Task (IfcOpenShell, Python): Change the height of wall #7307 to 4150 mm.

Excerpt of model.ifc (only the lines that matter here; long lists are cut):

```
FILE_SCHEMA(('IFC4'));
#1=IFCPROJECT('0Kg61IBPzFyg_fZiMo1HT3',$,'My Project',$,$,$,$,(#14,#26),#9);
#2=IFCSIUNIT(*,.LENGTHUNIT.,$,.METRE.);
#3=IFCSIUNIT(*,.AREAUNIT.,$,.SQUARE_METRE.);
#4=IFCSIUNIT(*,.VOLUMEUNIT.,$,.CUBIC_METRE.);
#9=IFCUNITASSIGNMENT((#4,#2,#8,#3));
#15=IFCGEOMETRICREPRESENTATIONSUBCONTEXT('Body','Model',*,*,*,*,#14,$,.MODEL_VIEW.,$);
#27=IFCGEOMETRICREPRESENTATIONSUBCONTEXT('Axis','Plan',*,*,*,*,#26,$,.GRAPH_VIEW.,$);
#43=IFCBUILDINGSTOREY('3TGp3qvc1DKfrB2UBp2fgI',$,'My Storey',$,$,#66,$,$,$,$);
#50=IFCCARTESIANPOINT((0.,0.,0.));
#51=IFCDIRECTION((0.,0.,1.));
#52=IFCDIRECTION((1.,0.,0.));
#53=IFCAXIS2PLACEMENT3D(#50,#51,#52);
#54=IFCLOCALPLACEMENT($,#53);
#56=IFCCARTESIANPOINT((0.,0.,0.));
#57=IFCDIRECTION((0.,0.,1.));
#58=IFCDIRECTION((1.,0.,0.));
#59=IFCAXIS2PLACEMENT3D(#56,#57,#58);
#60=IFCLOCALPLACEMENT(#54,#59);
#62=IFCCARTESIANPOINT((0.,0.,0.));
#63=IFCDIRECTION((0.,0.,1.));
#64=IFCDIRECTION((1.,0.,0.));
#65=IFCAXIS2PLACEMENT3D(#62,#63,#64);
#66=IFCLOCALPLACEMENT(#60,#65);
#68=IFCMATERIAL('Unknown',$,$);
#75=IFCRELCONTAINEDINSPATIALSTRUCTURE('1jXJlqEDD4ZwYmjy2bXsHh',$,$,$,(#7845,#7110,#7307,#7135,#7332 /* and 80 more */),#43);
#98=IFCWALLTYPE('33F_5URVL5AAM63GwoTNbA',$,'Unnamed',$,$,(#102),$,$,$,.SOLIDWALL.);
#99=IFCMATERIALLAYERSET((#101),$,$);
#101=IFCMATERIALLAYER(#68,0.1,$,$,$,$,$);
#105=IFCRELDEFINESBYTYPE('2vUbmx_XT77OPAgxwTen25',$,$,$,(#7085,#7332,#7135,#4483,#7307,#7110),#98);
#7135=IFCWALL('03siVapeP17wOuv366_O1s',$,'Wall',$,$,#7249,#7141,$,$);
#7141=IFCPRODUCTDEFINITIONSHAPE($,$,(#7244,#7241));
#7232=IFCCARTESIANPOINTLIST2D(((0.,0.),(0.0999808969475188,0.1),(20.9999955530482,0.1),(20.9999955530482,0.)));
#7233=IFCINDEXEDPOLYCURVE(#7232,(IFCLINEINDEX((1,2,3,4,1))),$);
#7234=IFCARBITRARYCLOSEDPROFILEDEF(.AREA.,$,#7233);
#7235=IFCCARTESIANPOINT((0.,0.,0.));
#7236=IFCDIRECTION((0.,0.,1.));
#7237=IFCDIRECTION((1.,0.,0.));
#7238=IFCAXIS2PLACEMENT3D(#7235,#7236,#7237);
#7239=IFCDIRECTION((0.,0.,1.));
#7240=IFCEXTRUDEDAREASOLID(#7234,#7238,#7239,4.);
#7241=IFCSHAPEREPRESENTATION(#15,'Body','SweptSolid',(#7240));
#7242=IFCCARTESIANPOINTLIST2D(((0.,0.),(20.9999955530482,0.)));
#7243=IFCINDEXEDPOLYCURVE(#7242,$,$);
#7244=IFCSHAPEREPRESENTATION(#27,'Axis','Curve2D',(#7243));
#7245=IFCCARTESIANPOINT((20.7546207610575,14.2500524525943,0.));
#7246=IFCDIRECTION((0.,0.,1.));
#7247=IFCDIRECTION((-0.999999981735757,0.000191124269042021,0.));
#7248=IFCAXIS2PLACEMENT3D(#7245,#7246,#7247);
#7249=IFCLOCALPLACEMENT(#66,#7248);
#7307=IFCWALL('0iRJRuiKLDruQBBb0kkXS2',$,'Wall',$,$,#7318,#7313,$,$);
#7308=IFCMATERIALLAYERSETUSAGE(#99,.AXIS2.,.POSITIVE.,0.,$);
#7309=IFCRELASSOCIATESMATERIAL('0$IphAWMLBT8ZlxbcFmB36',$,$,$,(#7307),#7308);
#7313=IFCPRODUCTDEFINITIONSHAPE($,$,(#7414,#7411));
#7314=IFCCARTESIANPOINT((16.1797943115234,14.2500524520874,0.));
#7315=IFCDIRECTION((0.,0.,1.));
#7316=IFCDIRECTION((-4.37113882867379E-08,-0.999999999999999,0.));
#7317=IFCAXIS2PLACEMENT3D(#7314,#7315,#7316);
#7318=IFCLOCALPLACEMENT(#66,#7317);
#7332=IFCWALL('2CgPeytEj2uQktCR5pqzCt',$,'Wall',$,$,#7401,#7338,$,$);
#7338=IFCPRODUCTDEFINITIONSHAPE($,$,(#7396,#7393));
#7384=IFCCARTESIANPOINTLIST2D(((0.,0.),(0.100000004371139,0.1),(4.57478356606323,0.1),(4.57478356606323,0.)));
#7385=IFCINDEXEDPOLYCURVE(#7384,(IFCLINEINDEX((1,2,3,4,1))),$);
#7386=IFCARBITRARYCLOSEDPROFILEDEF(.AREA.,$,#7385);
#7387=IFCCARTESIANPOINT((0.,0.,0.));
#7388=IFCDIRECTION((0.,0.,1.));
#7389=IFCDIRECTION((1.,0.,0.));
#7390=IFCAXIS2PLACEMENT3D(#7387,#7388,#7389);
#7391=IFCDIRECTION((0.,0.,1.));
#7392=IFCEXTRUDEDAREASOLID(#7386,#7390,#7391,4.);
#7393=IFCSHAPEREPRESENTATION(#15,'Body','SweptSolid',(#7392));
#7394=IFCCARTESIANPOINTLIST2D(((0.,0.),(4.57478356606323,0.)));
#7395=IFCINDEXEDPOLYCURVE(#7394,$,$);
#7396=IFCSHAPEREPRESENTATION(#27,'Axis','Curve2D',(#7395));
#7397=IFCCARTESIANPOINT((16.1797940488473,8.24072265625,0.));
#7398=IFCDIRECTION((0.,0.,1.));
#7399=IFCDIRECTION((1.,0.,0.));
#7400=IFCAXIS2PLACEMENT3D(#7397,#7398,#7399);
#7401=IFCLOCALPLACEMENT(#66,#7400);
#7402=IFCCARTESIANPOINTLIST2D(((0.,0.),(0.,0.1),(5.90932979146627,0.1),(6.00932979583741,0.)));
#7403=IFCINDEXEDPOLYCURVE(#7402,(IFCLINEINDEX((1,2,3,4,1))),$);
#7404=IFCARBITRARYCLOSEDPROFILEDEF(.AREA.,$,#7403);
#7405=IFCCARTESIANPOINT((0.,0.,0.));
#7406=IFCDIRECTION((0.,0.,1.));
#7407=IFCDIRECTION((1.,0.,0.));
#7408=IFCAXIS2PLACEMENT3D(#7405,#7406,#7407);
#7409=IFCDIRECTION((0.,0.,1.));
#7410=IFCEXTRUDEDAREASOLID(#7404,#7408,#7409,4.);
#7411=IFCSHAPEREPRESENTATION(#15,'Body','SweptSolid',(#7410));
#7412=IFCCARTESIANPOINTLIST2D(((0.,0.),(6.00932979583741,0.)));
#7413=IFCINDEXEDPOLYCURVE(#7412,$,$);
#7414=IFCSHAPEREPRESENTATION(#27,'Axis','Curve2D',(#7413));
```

```python
import ifcopenshell
import ifcopenshell.geom
import ifcopenshell.util.representation
import ifcopenshell.util.shape
import ifcopenshell.util.unit

model = ifcopenshell.open("model.ifc")
unit_scale = ifcopenshell.util.unit.calculate_unit_scale(model)
settings = ifcopenshell.geom.settings()


def volume(element):
    """Net volume in cubic metres, openings subtracted."""
    shape = ifcopenshell.geom.create_shape(settings, element)
    return ifcopenshell.util.shape.get_volume(shape.geometry)


wall = model.by_guid("0iRJRuiKLDruQBBb0kkXS2")
before = volume(wall)

body = ifcopenshell.util.representation.get_representation(wall, "Model", "Body")
solid = body.Items[0]
old_height = solid.Depth
solid.Depth = 4.15 / unit_scale
after = volume(wall)

print(f"height {old_height:g} -> {solid.Depth:g}, volume {before:.3f} -> {after:.3f} m3")

model.write("model_edited.ifc")
```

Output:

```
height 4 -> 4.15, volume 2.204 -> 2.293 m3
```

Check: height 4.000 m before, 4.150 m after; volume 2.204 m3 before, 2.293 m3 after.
